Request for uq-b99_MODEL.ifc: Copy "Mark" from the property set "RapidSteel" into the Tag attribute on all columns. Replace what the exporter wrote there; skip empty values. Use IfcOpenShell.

First a look at what the model holds.

```python
import ifcopenshell
import ifcopenshell.util.element

model = ifcopenshell.open("uq-b99_MODEL.ifc")
print(model.schema)
columns = model.by_type("IfcColumn")
print(len(columns), "columns")
for e in columns[:8]:
    source = ifcopenshell.util.element.get_pset(e, "RapidSteel", "Mark")
    target = e.Tag
    print(e.id(), repr(source), repr(target), sep=" | ")
```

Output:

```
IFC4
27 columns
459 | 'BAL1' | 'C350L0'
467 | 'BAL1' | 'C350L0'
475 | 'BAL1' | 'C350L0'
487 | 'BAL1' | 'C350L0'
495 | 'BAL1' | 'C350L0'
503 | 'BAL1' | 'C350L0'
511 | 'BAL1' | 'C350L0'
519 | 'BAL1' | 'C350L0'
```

```python
import ifcopenshell
import ifcopenshell.util.element

model = ifcopenshell.open("uq-b99_MODEL.ifc")

count = 0
for e in model.by_type("IfcColumn"):
    value = ifcopenshell.util.element.get_pset(e, "RapidSteel", "Mark")
    current = e.Tag
    if not value or not value.strip() or current == value:
        continue
    e.Tag = value
    count += 1

print(count, "columns updated")

model.write("uq-b99_MODEL_updated.ifc")
```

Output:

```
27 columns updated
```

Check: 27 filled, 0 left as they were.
